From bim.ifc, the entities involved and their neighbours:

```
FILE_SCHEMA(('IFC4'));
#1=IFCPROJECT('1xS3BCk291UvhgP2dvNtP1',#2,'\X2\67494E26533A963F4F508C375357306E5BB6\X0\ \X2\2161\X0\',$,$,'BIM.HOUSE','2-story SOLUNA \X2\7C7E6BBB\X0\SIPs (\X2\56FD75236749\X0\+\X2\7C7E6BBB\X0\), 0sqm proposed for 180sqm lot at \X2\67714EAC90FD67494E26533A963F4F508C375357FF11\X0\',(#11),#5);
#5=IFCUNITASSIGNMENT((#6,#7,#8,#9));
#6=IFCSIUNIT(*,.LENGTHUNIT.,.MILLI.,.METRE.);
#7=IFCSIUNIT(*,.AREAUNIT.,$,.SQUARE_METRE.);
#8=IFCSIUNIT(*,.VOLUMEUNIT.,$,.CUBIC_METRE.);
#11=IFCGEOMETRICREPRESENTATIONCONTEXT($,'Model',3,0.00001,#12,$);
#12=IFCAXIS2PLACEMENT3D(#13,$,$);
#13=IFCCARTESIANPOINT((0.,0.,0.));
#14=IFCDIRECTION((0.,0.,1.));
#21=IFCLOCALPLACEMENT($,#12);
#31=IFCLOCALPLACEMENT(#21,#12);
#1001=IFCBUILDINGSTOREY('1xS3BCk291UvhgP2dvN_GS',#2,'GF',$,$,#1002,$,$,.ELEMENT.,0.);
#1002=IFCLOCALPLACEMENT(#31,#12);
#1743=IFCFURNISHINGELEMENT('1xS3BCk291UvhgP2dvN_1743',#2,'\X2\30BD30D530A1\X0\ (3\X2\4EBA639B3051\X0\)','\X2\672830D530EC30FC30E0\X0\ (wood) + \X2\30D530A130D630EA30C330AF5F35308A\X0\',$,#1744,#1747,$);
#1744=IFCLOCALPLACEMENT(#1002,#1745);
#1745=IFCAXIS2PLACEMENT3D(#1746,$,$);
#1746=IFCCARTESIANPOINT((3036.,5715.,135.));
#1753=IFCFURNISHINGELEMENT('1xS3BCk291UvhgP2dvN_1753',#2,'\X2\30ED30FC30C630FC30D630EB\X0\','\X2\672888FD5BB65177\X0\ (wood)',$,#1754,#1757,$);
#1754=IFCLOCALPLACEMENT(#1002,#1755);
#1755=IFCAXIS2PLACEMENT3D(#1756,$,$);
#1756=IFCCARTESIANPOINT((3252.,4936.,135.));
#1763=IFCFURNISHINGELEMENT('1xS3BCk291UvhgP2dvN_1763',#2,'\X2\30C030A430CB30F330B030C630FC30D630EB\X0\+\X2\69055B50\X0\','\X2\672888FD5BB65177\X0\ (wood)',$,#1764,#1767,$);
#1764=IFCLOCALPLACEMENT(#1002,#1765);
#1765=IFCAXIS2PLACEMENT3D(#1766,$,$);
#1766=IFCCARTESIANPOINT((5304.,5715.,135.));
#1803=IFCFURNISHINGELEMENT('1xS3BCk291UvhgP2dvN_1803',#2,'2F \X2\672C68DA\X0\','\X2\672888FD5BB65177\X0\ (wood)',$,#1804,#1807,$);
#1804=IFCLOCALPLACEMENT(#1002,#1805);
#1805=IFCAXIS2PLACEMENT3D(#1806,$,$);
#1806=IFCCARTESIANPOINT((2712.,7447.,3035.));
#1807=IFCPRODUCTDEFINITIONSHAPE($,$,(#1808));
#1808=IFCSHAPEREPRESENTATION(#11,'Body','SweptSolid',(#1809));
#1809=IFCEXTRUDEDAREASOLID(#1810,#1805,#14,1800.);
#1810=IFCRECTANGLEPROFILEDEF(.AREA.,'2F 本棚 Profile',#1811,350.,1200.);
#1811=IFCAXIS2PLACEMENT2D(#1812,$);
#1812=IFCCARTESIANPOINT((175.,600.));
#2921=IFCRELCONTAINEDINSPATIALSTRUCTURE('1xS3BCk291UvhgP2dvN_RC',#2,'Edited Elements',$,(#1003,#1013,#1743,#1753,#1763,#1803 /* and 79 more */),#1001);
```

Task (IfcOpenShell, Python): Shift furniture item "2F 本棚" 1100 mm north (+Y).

```python
import ifcopenshell
import ifcopenshell.api.geometry
import ifcopenshell.util.placement
import ifcopenshell.util.unit

model = ifcopenshell.open("bim.ifc")
unit_scale = ifcopenshell.util.unit.calculate_unit_scale(model)

item = model.by_guid("1xS3BCk291UvhgP2dvN_1803")
matrix = ifcopenshell.util.placement.get_local_placement(item.ObjectPlacement)
matrix[1, 3] += 1.1 / unit_scale
ifcopenshell.api.geometry.edit_object_placement(model, product=item, matrix=matrix, is_si=False)

print(ifcopenshell.util.placement.get_local_placement(item.ObjectPlacement).round(3) + 0.0)

model.write("bim_edited.ifc")
```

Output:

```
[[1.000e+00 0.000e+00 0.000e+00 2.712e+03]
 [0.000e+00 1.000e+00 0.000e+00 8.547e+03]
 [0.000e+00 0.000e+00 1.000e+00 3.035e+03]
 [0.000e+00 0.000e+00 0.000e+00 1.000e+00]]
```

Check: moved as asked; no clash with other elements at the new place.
